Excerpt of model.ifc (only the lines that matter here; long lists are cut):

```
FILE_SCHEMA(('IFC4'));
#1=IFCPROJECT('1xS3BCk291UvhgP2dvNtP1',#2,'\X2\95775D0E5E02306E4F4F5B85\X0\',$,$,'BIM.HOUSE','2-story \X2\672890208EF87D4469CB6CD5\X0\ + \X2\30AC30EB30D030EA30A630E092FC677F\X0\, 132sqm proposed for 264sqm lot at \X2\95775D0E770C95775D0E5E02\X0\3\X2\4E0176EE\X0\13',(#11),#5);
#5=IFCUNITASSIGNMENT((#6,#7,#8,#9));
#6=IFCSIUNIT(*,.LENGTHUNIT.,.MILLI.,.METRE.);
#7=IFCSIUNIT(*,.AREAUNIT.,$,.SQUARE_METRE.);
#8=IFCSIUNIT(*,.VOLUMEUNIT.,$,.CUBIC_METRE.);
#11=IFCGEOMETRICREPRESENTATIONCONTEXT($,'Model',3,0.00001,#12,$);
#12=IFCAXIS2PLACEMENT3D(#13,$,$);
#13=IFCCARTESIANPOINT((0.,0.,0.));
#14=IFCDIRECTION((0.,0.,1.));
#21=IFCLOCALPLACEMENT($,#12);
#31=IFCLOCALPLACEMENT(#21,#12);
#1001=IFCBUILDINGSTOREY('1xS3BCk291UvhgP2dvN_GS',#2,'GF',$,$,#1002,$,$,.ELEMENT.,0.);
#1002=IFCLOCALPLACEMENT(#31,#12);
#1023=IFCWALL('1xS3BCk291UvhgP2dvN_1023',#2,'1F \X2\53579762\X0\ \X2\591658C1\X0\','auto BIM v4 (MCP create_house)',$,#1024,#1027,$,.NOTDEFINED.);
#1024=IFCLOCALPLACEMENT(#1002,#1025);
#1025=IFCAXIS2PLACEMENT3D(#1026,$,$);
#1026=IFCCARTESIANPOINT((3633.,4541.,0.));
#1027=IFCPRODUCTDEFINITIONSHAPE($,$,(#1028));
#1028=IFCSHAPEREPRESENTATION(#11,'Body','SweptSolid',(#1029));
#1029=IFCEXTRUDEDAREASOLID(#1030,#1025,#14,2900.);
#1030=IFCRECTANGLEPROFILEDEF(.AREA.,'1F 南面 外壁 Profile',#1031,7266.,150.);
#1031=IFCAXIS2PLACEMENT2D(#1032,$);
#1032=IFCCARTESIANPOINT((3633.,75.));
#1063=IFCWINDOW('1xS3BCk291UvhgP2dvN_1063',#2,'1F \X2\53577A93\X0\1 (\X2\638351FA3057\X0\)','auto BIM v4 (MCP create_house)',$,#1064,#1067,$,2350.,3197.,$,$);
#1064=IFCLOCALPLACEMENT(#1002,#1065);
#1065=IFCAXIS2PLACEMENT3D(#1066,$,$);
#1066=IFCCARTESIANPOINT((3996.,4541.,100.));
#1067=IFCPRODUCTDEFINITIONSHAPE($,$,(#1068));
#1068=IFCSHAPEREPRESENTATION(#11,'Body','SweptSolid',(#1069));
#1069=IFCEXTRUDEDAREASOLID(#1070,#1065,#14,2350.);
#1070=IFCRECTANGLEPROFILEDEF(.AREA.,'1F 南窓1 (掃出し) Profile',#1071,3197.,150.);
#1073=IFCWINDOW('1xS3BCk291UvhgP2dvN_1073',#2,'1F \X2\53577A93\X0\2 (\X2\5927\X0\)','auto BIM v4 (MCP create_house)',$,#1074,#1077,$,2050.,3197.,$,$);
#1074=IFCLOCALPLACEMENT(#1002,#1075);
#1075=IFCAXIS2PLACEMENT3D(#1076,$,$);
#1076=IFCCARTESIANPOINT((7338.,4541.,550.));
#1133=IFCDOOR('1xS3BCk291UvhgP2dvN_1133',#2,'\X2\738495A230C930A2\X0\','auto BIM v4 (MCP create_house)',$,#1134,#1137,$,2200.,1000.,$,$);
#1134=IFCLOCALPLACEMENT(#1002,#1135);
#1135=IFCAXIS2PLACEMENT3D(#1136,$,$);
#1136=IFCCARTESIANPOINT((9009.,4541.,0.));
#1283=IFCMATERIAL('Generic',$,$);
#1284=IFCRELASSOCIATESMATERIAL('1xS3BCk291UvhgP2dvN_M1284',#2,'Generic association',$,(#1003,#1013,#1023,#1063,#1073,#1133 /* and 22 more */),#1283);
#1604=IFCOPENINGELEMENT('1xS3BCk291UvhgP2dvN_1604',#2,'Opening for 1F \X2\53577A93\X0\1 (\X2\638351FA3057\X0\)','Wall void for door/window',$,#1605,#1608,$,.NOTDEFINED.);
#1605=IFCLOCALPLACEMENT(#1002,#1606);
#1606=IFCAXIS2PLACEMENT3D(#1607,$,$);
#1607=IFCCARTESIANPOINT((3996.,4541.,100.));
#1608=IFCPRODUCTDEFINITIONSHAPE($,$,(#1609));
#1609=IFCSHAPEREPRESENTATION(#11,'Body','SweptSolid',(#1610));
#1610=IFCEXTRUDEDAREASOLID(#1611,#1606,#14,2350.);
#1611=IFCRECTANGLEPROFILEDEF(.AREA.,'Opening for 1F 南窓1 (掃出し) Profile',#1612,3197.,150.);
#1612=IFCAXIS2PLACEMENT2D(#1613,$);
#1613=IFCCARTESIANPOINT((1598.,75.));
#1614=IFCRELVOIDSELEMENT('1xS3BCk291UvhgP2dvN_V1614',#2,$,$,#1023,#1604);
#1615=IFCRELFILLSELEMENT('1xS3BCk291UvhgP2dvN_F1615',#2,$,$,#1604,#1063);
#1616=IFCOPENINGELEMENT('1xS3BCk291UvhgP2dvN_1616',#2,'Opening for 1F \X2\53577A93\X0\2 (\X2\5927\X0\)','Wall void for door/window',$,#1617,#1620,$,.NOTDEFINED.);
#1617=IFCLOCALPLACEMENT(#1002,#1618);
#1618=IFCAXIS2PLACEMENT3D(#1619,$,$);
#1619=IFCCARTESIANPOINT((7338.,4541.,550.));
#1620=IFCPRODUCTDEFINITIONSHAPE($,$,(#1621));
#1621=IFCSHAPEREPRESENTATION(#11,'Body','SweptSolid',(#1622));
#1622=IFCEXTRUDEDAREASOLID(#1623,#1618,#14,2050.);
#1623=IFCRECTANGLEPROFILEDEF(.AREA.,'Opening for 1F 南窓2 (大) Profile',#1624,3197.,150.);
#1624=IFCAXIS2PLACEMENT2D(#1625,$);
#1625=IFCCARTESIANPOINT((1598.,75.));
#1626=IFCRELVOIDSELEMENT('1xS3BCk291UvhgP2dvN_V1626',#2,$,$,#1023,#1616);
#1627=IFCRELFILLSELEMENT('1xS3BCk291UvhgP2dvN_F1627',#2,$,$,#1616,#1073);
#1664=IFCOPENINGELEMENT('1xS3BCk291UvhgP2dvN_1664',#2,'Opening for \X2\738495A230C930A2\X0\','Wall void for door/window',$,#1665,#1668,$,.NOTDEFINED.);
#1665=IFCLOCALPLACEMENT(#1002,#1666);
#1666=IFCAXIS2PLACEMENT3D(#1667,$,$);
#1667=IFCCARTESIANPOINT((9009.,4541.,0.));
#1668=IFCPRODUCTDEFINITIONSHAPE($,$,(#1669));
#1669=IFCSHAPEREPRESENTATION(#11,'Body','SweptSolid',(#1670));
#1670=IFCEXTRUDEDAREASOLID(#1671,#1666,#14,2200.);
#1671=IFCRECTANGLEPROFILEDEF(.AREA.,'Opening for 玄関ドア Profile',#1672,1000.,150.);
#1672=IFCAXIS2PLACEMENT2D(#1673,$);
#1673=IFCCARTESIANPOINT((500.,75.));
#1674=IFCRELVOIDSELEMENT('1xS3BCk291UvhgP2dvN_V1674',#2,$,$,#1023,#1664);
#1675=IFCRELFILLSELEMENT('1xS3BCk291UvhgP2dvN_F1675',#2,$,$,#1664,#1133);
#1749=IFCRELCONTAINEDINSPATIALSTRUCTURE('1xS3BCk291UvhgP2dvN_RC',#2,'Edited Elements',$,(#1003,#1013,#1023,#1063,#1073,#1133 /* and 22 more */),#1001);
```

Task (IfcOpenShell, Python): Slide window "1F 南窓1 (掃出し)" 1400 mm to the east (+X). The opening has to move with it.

```python
import ifcopenshell
import ifcopenshell.api.geometry
import ifcopenshell.util.placement
import ifcopenshell.util.unit

model = ifcopenshell.open("model.ifc")
unit_scale = ifcopenshell.util.unit.calculate_unit_scale(model)

window = model.by_guid("1xS3BCk291UvhgP2dvN_1063")
opening = window.FillsVoids[0].RelatingOpeningElement
wall = opening.VoidsElements[0].RelatingBuildingElement

wall_matrix = ifcopenshell.util.placement.get_local_placement(wall.ObjectPlacement)
shift = wall_matrix[:3, 0] * 1.4 / unit_scale
before = ifcopenshell.util.placement.get_local_placement(window.ObjectPlacement)[:3, 3].copy()

# The window is not placed relative to its opening, so move both.
for product in (opening, window):
    matrix = ifcopenshell.util.placement.get_local_placement(product.ObjectPlacement)
    matrix[:3, 3] += shift
    ifcopenshell.api.geometry.edit_object_placement(model, product=product, matrix=matrix, is_si=False)

after = ifcopenshell.util.placement.get_local_placement(window.ObjectPlacement)[:3, 3]
print("window moved by", (after - before).round(3) + 0.0)

model.write("model-out.ifc")
```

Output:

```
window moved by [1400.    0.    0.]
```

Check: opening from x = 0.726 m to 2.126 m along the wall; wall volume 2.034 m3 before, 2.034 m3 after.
